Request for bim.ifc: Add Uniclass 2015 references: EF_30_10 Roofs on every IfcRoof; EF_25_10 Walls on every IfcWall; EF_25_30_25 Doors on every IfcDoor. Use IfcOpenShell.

First a look at what the model holds.

```python
import ifcopenshell

model = ifcopenshell.open("bim.ifc")
print(model.schema)
print("classifications:", [c.Name for c in model.by_type("IfcClassification")])
for ifc_class in ("IfcDoor", "IfcRoof", "IfcStair", "IfcWall", "IfcWindow"):
    print(ifc_class, len(model.by_type(ifc_class)))
```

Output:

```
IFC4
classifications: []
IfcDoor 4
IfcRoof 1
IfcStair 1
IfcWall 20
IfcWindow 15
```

```python
import ifcopenshell
import ifcopenshell.api.classification

model = ifcopenshell.open("bim.ifc")

system = ifcopenshell.api.classification.add_classification(model, classification="Uniclass 2015")

codes = {
    "IfcRoof": ("EF_30_10", "Roofs"),
    "IfcWall": ("EF_25_10", "Walls"),
    "IfcDoor": ("EF_25_30_25", "Doors"),
}
for ifc_class, (code, name) in codes.items():
    products = model.by_type(ifc_class)
    ifcopenshell.api.classification.add_reference(
        model, products=products, classification=system, identification=code, name=name
    )
    print(code, len(products))

model.write("bim_rev.ifc")
```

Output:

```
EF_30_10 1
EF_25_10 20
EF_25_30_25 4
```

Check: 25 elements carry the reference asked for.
